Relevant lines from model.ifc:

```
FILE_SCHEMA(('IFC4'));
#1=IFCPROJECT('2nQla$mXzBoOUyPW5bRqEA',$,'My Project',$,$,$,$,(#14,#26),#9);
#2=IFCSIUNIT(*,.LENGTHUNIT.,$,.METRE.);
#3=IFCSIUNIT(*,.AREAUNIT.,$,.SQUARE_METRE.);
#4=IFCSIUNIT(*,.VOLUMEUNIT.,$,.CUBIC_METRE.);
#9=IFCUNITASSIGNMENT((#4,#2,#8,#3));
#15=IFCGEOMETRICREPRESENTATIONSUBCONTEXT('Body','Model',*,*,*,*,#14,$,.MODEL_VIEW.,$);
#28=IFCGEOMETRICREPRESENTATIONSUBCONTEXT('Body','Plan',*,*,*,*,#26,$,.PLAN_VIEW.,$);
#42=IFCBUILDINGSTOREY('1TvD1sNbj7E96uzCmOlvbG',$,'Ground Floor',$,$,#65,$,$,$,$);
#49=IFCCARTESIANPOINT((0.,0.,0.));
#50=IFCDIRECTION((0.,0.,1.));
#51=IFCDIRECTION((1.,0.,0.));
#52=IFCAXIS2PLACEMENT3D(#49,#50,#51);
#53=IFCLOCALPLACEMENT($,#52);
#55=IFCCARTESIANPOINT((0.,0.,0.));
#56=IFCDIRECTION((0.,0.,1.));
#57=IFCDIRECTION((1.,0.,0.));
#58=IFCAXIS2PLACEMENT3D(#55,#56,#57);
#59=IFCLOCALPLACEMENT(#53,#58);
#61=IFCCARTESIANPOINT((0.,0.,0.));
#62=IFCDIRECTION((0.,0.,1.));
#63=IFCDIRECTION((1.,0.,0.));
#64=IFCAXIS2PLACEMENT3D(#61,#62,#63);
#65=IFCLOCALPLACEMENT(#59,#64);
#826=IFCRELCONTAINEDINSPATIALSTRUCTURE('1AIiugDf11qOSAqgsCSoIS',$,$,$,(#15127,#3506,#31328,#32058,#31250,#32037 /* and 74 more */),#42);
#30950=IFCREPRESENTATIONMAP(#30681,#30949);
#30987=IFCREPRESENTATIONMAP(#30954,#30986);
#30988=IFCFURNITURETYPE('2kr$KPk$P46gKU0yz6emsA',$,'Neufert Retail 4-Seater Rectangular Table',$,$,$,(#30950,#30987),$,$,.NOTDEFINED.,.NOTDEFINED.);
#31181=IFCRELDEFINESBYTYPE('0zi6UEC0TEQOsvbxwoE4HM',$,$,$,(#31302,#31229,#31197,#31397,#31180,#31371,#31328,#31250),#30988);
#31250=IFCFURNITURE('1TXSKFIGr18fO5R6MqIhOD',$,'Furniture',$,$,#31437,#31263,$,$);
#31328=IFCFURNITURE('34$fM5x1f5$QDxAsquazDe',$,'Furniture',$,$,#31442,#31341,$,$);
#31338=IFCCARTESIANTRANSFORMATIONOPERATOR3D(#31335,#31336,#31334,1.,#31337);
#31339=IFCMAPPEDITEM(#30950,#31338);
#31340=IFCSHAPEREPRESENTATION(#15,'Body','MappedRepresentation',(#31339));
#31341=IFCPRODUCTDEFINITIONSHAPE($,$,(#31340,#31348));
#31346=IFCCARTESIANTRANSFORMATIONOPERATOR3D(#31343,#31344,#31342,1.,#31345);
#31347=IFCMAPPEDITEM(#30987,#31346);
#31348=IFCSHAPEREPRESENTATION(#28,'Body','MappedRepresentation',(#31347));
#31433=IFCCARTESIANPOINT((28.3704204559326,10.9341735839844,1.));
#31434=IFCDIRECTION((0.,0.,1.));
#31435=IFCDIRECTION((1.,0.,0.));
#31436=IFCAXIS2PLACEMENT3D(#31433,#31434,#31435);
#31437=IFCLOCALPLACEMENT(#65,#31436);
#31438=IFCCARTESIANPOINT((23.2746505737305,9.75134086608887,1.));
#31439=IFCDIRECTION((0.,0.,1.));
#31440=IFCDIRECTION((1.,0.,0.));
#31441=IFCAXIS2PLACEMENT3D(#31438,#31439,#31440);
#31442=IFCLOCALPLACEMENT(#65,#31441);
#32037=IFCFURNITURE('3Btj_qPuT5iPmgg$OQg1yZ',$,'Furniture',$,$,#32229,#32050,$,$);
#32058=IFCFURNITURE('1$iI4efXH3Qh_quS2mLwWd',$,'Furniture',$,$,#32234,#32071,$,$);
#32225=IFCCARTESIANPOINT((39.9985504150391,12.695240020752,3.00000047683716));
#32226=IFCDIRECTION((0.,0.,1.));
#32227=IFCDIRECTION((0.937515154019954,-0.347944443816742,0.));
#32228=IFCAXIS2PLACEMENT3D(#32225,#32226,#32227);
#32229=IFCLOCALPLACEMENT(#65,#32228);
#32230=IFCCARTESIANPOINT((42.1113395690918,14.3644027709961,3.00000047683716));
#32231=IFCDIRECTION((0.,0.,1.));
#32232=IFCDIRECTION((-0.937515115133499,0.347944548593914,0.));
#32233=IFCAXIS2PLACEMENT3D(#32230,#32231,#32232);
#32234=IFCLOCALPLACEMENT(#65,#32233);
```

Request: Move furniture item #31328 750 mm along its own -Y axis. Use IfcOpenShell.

```python
import ifcopenshell
import ifcopenshell.api.geometry
import ifcopenshell.util.placement
import ifcopenshell.util.unit

model = ifcopenshell.open("model.ifc")
unit_scale = ifcopenshell.util.unit.calculate_unit_scale(model)

item = model.by_id(31328)
matrix = ifcopenshell.util.placement.get_local_placement(item.ObjectPlacement)
matrix[:3, 3] -= matrix[:3, 1] * 0.75 / unit_scale
ifcopenshell.api.geometry.edit_object_placement(model, product=item, matrix=matrix, is_si=False)

print(ifcopenshell.util.placement.get_local_placement(item.ObjectPlacement).round(3) + 0.0)

model.write("model_v2.ifc")
```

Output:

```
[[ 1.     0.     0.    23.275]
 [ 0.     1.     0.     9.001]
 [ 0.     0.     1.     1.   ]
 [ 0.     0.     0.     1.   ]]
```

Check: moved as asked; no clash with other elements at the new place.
